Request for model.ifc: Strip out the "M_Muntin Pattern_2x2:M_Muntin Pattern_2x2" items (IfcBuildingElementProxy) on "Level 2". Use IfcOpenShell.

First a look at what the model holds.

```python
import ifcopenshell
import ifcopenshell.util.element

model = ifcopenshell.open("model.ifc")
print(model.schema)
storey = next(s for s in model.by_type("IfcBuildingStorey") if s.Name == "Level 2")
proxies = [e for e in ifcopenshell.util.element.get_decomposition(storey) if e.is_a("IfcBuildingElementProxy")]
seen = {}
for e in proxies:
    element_type = ifcopenshell.util.element.get_type(e)
    name = element_type.Name if element_type not in (None, e) else None
    seen[name] = seen.get(name, 0) + 1
for name, count in sorted(seen.items(), key=str):
    print(count, "x", name)
```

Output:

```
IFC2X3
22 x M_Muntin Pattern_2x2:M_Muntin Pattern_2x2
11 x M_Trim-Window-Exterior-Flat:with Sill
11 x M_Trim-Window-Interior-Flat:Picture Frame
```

```python
import ifcopenshell
import ifcopenshell.api.root
import ifcopenshell.util.element

model = ifcopenshell.open("model.ifc")

storey = next(s for s in model.by_type("IfcBuildingStorey") if s.Name == "Level 2")
proxies = [e for e in ifcopenshell.util.element.get_decomposition(storey) if e.is_a("IfcBuildingElementProxy")]
targets = [e for e in proxies if (t := ifcopenshell.util.element.get_type(e)) not in (None, e) and t.Name == "M_Muntin Pattern_2x2:M_Muntin Pattern_2x2"]

for e in targets:
    ifcopenshell.api.root.remove_product(model, product=e)
print(len(targets), "removed")

model.write("model_v2.ifc")
```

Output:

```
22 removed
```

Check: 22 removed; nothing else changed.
